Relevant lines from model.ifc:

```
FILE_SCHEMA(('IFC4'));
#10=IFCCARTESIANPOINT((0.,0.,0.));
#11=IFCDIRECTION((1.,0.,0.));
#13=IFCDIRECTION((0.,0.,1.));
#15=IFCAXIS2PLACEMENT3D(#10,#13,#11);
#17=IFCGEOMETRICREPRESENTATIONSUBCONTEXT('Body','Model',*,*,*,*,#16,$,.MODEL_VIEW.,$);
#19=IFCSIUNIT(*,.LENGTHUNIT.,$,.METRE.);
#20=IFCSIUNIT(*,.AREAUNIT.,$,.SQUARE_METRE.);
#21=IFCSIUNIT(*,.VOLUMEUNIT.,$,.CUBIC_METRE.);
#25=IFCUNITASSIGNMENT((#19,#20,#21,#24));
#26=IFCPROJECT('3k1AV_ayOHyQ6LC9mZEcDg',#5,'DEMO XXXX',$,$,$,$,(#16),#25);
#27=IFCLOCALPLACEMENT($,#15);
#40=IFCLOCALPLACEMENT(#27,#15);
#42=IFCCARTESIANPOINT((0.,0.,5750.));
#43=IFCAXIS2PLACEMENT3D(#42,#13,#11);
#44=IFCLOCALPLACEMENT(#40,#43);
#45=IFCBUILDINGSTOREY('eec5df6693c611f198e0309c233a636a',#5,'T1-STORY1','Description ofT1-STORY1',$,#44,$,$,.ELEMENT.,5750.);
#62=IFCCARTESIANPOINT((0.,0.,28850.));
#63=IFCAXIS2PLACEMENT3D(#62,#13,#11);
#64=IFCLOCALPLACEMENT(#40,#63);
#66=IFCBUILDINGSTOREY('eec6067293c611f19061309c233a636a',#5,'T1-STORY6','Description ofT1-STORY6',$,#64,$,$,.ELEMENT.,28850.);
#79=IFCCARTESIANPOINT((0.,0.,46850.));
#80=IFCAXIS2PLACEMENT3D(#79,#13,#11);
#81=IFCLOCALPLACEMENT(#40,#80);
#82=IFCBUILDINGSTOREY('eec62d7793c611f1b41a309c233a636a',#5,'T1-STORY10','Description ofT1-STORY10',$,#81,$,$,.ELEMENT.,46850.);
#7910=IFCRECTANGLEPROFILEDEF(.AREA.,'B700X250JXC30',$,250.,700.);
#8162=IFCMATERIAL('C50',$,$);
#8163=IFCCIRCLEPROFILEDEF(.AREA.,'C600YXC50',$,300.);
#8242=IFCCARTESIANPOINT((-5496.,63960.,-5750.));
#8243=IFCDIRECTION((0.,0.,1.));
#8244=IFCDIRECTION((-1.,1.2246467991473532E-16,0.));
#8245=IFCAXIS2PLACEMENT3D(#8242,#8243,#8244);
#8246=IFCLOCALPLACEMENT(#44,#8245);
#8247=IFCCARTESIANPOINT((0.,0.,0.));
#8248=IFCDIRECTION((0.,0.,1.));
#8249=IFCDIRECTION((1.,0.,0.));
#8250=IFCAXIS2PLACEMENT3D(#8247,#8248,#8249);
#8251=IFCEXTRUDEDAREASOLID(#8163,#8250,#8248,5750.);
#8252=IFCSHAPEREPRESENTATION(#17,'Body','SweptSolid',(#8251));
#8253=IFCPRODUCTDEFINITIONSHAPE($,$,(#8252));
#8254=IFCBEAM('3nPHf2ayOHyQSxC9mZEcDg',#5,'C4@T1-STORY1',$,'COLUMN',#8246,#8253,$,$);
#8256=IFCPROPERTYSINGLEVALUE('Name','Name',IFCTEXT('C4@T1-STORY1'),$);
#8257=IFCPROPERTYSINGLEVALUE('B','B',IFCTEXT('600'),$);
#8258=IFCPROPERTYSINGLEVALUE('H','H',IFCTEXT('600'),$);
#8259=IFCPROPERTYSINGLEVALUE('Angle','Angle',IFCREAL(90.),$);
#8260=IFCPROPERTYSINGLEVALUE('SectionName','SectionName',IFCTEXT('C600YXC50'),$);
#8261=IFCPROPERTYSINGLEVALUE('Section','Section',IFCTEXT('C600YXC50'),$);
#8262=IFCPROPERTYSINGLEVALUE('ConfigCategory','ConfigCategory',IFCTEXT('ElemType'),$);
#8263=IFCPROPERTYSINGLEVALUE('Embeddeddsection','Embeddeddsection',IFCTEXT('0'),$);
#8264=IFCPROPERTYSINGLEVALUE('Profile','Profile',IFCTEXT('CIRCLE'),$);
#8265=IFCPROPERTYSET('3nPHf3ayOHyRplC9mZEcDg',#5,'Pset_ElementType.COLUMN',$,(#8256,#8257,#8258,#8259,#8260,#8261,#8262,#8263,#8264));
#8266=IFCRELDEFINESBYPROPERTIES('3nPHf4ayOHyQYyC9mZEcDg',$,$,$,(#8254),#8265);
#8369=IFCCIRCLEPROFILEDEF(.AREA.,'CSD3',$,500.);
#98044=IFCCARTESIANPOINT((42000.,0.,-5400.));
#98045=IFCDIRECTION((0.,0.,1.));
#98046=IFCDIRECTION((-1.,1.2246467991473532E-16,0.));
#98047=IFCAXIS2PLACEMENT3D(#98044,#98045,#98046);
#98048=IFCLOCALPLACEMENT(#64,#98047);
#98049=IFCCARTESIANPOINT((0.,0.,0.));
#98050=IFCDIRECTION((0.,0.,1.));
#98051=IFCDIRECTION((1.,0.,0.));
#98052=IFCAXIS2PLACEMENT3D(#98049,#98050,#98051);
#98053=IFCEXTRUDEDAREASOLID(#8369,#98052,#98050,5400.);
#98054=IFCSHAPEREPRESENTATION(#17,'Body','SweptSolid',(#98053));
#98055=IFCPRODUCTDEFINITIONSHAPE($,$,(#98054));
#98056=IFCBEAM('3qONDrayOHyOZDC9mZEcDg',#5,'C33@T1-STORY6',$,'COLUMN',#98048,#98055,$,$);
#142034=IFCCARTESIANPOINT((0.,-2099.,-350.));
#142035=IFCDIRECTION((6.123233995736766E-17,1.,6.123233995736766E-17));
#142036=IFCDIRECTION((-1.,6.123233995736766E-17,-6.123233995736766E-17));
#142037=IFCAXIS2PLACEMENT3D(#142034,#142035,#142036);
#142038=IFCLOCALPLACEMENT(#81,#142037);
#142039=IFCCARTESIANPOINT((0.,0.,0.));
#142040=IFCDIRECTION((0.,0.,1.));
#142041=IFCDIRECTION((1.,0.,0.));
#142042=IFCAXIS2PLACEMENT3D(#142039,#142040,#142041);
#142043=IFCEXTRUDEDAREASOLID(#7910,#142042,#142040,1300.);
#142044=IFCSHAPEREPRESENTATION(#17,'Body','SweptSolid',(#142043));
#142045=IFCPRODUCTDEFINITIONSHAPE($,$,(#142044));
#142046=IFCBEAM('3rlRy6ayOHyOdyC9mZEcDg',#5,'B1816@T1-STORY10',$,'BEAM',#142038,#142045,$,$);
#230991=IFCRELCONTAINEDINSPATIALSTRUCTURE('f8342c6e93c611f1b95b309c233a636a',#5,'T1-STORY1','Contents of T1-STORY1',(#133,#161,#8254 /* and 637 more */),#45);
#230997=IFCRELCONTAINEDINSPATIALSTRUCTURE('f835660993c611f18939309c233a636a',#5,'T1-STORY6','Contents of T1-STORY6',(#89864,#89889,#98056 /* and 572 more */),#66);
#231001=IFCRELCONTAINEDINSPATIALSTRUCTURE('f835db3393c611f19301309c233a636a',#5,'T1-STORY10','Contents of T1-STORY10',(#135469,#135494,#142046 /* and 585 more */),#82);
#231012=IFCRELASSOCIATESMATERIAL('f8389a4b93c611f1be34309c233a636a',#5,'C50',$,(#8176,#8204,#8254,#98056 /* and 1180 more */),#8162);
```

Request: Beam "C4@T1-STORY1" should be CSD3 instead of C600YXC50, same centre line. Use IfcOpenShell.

```python
import ifcopenshell
import ifcopenshell.api.pset
import ifcopenshell.util.element
import ifcopenshell.util.representation

model = ifcopenshell.open("model.ifc")

member = model.by_id(8254)
source = next(p for p in model.by_type("IfcCircleProfileDef") if p.ProfileName == "CSD3")

body = ifcopenshell.util.representation.get_representation(member, "Model", "Body")
solid = body.Items[0]
old_profile = solid.SweptArea

# Copy the section's sizes but keep this member's own profile position.
profile = ifcopenshell.util.element.copy(model, source)
profile.Position = old_profile.Position
solid.SweptArea = profile
if not model.get_total_inverses(old_profile):
    ifcopenshell.util.element.remove_deep2(model, old_profile)
pset = model.by_id(ifcopenshell.util.element.get_pset(member, "Pset_ElementType.COLUMN", should_inherit=False)["id"])
ifcopenshell.api.pset.edit_pset(model, pset=pset, properties={"SectionName": "CSD3"})
pset = model.by_id(ifcopenshell.util.element.get_pset(member, "Pset_ElementType.COLUMN", should_inherit=False)["id"])
ifcopenshell.api.pset.edit_pset(model, pset=pset, properties={"Section": "CSD3"})

print(solid.SweptArea)

model.write("model_rev.ifc")
```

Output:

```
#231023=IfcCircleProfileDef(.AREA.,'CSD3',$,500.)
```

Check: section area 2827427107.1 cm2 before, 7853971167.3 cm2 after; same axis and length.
